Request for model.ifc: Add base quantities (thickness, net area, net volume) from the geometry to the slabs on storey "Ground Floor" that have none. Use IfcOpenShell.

First a look at what the model holds.

```python
import ifcopenshell
import ifcopenshell.util.element
import ifcopenshell.util.unit

model = ifcopenshell.open("model.ifc")
print(model.schema)
for unit_type in ("LENGTHUNIT", "AREAUNIT", "VOLUMEUNIT"):
    print(unit_type, ifcopenshell.util.unit.calculate_unit_scale(model, unit_type))
storey = next(s for s in model.by_type("IfcBuildingStorey") if s.Name == "Ground Floor")
slabs = [e for e in ifcopenshell.util.element.get_decomposition(storey) if e.is_a("IfcSlab")]
for e in sorted(slabs, key=lambda e: e.id()):
    print(e.id(), e.is_a(), e.Name, list(ifcopenshell.util.element.get_psets(e, qtos_only=True)), sep=" | ")
```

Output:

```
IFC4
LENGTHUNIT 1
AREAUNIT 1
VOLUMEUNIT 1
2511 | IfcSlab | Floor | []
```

```python
import ifcopenshell
import ifcopenshell.api.pset
import ifcopenshell.geom
import ifcopenshell.util.element
import ifcopenshell.util.shape
import ifcopenshell.util.unit

model = ifcopenshell.open("model.ifc")
unit_scale = ifcopenshell.util.unit.calculate_unit_scale(model)
area_scale = ifcopenshell.util.unit.calculate_unit_scale(model, "AREAUNIT")
volume_scale = ifcopenshell.util.unit.calculate_unit_scale(model, "VOLUMEUNIT")
settings = ifcopenshell.geom.settings()

storey = next(s for s in model.by_type("IfcBuildingStorey") if s.Name == "Ground Floor")
slabs = [e for e in ifcopenshell.util.element.get_decomposition(storey) if e.is_a("IfcSlab")]

for e in sorted(slabs, key=lambda e: e.id()):
    if ifcopenshell.util.element.get_psets(e, qtos_only=True, should_inherit=False):
        continue
    # Geometry comes back in metres, in the element's own axes.
    shape = ifcopenshell.geom.create_shape(settings, e)
    values = {
        "Width": ifcopenshell.util.shape.get_z(shape.geometry) / unit_scale,
        "NetArea": ifcopenshell.util.shape.get_footprint_area(shape.geometry) / area_scale,
        "NetVolume": ifcopenshell.util.shape.get_volume(shape.geometry) / volume_scale,
    }
    qto = ifcopenshell.api.pset.add_qto(model, product=e, name="Qto_SlabBaseQuantities")
    ifcopenshell.api.pset.edit_qto(model, qto=qto, properties=values)
    print(e.id(), {k: round(v, 3) for k, v in values.items()})

model.write("model_v2.ifc")
```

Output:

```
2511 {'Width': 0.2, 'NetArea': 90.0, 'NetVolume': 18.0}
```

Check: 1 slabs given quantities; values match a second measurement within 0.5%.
